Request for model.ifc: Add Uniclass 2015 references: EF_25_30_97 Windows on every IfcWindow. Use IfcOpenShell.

First a look at what the model holds.

```python
import ifcopenshell

model = ifcopenshell.open("model.ifc")
print(model.schema)
print("classifications:", [c.Name for c in model.by_type("IfcClassification")])
for ifc_class in ("IfcDoor", "IfcRoof", "IfcStair", "IfcWall", "IfcWindow"):
    print(ifc_class, len(model.by_type(ifc_class)))
```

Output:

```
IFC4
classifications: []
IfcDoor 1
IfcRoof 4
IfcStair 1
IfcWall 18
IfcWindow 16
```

```python
import ifcopenshell
import ifcopenshell.api.classification

model = ifcopenshell.open("model.ifc")

system = ifcopenshell.api.classification.add_classification(model, classification="Uniclass 2015")

codes = {
    "IfcWindow": ("EF_25_30_97", "Windows"),
}
for ifc_class, (code, name) in codes.items():
    products = model.by_type(ifc_class)
    ifcopenshell.api.classification.add_reference(
        model, products=products, classification=system, identification=code, name=name
    )
    print(code, len(products))

model.write("model_v2.ifc")
```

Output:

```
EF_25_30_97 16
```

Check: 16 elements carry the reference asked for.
